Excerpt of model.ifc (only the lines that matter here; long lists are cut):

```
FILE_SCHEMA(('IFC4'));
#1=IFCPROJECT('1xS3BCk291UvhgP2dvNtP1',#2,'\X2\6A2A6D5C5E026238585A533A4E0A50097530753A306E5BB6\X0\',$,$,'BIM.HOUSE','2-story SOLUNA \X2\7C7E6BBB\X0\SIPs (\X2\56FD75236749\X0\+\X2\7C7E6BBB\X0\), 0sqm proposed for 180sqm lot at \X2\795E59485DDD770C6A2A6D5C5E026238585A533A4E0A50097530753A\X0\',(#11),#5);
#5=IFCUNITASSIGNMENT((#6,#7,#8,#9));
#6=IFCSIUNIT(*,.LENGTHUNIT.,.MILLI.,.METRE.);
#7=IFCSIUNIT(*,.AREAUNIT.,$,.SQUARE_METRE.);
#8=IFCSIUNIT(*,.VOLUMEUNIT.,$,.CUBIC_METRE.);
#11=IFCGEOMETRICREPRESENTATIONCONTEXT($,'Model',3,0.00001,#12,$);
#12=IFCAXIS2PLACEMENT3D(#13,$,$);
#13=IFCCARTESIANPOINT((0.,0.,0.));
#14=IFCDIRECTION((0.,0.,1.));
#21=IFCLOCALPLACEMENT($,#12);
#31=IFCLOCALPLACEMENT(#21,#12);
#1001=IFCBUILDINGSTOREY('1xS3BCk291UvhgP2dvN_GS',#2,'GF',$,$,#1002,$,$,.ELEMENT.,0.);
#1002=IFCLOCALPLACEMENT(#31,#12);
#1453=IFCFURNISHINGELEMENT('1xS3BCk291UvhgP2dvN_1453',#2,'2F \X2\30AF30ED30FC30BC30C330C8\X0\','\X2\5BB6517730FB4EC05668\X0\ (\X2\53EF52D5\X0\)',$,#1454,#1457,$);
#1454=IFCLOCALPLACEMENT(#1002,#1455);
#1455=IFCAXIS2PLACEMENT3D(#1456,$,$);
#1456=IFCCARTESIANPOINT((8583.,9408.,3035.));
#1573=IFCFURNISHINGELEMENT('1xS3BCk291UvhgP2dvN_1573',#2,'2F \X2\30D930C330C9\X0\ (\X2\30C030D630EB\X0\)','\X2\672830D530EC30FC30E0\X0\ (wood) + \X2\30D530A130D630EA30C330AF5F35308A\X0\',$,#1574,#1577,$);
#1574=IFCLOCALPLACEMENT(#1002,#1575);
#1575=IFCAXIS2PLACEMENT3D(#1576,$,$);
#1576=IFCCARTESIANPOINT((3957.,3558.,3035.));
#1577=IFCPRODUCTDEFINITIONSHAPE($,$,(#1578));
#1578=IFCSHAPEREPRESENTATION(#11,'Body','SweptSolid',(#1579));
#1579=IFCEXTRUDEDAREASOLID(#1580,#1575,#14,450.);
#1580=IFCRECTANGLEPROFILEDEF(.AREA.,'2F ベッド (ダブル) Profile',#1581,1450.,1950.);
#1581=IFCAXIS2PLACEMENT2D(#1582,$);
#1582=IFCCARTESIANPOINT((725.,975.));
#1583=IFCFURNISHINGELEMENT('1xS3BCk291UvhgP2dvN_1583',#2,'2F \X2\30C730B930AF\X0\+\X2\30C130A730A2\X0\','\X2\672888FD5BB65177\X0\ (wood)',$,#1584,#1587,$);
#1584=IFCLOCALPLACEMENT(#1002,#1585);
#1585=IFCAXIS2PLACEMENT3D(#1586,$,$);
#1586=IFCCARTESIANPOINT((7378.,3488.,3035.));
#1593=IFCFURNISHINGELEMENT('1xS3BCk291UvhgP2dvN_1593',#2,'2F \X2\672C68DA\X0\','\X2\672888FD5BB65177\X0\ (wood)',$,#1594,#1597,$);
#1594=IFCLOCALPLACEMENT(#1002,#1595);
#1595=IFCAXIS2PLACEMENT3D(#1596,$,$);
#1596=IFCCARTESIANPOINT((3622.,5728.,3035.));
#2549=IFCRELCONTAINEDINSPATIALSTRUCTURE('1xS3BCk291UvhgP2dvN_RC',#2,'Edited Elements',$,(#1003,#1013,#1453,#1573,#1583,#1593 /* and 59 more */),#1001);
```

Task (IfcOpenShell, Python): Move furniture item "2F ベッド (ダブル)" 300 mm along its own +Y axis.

```python
import ifcopenshell
import ifcopenshell.api.geometry
import ifcopenshell.util.placement
import ifcopenshell.util.unit

model = ifcopenshell.open("model.ifc")
unit_scale = ifcopenshell.util.unit.calculate_unit_scale(model)

item = model.by_guid("1xS3BCk291UvhgP2dvN_1573")
matrix = ifcopenshell.util.placement.get_local_placement(item.ObjectPlacement)
matrix[:3, 3] += matrix[:3, 1] * 0.3 / unit_scale
ifcopenshell.api.geometry.edit_object_placement(model, product=item, matrix=matrix, is_si=False)

print(ifcopenshell.util.placement.get_local_placement(item.ObjectPlacement).round(3) + 0.0)

model.write("model_rev.ifc")
```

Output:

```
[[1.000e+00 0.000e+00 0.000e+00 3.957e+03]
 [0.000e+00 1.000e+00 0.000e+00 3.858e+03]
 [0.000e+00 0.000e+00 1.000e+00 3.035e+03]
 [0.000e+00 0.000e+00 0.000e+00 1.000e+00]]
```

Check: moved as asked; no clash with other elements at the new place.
